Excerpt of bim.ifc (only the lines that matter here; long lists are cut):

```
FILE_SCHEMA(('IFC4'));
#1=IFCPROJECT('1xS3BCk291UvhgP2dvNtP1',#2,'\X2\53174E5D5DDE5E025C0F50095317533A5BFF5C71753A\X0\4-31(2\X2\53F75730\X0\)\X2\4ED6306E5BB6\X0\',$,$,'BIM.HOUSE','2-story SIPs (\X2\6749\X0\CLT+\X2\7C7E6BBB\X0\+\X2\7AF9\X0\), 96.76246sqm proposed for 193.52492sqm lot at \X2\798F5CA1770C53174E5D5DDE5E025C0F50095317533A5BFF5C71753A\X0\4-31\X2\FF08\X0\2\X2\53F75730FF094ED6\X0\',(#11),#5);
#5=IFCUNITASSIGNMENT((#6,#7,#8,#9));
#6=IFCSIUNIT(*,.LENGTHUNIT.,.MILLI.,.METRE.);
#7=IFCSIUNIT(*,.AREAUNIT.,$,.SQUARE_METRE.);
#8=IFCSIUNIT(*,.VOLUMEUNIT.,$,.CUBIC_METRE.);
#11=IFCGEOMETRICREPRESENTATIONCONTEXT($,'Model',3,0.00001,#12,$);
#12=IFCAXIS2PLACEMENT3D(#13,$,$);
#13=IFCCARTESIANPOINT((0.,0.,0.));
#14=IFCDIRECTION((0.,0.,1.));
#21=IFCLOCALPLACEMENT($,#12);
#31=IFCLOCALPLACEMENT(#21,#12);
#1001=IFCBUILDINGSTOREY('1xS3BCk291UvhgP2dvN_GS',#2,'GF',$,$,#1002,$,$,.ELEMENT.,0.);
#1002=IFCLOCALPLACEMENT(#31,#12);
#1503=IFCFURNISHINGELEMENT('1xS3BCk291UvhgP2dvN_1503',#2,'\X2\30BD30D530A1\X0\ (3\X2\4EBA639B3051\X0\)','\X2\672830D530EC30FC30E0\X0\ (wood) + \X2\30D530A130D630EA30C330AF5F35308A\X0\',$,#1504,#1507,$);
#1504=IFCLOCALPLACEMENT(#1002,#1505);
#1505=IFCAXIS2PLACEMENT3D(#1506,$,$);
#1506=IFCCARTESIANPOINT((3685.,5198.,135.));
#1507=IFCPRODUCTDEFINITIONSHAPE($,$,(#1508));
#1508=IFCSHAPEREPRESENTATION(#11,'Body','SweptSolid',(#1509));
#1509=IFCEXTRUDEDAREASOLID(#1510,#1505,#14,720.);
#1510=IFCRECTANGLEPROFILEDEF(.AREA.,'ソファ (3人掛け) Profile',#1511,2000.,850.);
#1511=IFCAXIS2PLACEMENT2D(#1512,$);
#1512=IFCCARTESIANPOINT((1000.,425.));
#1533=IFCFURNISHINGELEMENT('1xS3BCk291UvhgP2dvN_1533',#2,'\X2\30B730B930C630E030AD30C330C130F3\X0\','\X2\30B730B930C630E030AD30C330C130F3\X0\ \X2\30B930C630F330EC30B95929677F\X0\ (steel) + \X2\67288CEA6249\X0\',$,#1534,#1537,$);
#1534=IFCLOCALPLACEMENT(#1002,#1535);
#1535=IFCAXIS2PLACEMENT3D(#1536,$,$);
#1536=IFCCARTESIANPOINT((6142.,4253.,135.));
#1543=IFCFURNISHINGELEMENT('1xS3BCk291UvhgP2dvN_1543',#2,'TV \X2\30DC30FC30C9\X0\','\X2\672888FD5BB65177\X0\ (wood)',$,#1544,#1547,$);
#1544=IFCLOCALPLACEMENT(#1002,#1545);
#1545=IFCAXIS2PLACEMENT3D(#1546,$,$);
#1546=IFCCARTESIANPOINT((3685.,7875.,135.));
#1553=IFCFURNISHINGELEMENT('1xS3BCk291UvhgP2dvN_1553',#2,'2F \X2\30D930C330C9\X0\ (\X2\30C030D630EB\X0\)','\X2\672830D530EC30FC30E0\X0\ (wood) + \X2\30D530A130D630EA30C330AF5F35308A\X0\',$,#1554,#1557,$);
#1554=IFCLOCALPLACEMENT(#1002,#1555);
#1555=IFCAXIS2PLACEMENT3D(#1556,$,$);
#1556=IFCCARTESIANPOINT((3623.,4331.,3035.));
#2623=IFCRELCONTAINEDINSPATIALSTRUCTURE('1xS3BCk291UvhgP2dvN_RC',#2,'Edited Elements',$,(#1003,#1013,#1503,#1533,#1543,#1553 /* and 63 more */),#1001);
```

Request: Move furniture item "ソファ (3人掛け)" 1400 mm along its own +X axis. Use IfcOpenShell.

```python
import ifcopenshell
import ifcopenshell.api.geometry
import ifcopenshell.util.placement
import ifcopenshell.util.unit

model = ifcopenshell.open("bim.ifc")
unit_scale = ifcopenshell.util.unit.calculate_unit_scale(model)

item = model.by_id(1503)
matrix = ifcopenshell.util.placement.get_local_placement(item.ObjectPlacement)
matrix[:3, 3] += matrix[:3, 0] * 1.4 / unit_scale
ifcopenshell.api.geometry.edit_object_placement(model, product=item, matrix=matrix, is_si=False)

print(ifcopenshell.util.placement.get_local_placement(item.ObjectPlacement).round(3) + 0.0)

model.write("bim_v2.ifc")
```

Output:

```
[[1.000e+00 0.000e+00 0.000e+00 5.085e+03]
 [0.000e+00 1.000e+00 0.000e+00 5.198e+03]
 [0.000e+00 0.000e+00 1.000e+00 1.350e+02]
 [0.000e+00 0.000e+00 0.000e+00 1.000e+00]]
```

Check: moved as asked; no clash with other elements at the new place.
